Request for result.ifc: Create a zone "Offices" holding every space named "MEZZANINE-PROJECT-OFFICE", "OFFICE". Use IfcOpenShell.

First a look at what the model holds.

```python
import ifcopenshell

model = ifcopenshell.open("result.ifc")
print(model.schema)
seen = {}
for space in model.by_type("IfcSpace"):
    seen[space.Name] = seen.get(space.Name, 0) + 1
for name, count in sorted(seen.items(), key=str):
    print(count, "x", name)
print("zones:", [z.Name for z in model.by_type("IfcZone")][:20])
```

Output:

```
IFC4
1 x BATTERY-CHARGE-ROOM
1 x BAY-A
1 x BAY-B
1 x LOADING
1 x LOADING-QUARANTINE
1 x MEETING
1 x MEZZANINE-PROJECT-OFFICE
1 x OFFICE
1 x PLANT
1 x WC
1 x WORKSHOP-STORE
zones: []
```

```python
import ifcopenshell
import ifcopenshell.api.group
import ifcopenshell.api.root

model = ifcopenshell.open("result.ifc")

names = {"MEZZANINE-PROJECT-OFFICE", "OFFICE"}
spaces = [s for s in model.by_type("IfcSpace") if s.Name in names]

zone = ifcopenshell.api.root.create_entity(model, ifc_class="IfcZone", name="Offices")
ifcopenshell.api.group.assign_group(model, products=spaces, group=zone)
print(len(spaces), "spaces in", zone.Name)

model.write("result_edited.ifc")
```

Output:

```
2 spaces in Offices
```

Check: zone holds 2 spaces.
